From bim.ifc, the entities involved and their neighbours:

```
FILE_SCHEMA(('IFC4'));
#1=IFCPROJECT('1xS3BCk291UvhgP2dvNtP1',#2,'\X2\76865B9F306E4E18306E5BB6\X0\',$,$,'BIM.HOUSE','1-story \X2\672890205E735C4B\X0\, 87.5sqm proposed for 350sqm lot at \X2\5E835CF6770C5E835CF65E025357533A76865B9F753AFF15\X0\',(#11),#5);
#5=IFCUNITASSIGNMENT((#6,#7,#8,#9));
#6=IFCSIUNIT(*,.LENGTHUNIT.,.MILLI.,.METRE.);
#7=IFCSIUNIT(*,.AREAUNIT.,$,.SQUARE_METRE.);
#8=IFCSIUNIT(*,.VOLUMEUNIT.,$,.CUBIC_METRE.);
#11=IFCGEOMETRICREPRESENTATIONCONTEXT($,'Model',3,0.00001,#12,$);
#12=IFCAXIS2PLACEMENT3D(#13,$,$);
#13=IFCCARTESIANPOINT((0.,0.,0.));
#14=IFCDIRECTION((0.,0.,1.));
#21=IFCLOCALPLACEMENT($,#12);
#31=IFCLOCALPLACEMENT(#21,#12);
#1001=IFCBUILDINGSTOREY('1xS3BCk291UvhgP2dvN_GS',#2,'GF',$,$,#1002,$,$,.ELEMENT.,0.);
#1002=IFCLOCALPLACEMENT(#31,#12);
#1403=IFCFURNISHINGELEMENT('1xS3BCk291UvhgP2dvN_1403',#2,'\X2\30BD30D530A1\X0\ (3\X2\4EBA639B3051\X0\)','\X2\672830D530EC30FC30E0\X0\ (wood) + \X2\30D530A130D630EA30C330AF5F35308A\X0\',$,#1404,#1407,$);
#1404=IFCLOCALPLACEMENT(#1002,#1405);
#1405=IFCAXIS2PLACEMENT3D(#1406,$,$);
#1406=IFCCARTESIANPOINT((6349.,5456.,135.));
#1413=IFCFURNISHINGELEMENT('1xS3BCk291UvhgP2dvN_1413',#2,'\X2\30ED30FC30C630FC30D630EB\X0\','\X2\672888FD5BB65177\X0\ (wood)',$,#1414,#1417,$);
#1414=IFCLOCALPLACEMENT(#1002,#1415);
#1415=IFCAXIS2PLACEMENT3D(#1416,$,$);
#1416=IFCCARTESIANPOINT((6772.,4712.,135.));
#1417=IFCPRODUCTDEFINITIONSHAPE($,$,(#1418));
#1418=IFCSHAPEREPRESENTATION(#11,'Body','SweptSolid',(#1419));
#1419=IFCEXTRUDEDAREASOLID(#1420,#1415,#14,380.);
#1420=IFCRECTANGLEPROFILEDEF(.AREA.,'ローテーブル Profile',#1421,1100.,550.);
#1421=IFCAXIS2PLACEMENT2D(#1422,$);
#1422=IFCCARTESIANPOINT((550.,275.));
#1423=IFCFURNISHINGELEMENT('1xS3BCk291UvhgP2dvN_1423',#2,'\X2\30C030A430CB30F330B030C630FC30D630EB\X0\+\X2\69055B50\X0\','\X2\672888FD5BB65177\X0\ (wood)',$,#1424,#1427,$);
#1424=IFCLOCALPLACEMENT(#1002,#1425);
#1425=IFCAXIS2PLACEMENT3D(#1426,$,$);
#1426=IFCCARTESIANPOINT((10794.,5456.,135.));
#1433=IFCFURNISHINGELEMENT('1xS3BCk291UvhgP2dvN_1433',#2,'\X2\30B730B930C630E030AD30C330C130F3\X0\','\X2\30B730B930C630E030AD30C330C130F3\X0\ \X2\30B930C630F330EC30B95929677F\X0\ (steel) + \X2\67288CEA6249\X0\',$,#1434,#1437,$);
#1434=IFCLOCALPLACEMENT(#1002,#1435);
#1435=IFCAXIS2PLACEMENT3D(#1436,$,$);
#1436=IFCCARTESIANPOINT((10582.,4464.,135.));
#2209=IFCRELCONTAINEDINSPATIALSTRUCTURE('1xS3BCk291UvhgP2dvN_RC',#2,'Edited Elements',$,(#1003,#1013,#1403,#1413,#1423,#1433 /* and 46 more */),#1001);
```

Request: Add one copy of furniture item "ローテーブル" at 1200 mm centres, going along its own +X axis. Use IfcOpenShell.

```python
import ifcopenshell
import ifcopenshell.api.geometry
import ifcopenshell.api.root
import ifcopenshell.util.element
import ifcopenshell.util.placement

model = ifcopenshell.open("bim.ifc")


def reuse_history(source, copy):
    """copy_class also copies each property set's owner history, people and application; keep the originals."""
    for rel in copy.IsDefinedBy:
        if rel.is_a("IfcRelDefinesByProperties") and (history := rel.RelatingPropertyDefinition.OwnerHistory):
            rel.RelatingPropertyDefinition.OwnerHistory = source.OwnerHistory
            ifcopenshell.util.element.remove_deep2(model, history)


source = model.by_guid("1xS3BCk291UvhgP2dvN_1413")
base = ifcopenshell.util.placement.get_local_placement(source.ObjectPlacement)
step = base[:3, 0] * 1200.0

for i in range(1, 2):
    copy = ifcopenshell.api.root.copy_class(model, product=source)
    copy.Representation = ifcopenshell.util.element.copy_deep(
        model, source.Representation, exclude=["IfcGeometricRepresentationContext", "IfcRepresentationMap"]
    )
    reuse_history(source, copy)
    matrix = base.copy()
    matrix[:3, 3] += i * step
    print("added at", matrix[:3, 3].round(3) + 0.0)
    ifcopenshell.api.geometry.edit_object_placement(model, product=copy, matrix=matrix, is_si=False)

model.write("bim_rev.ifc")
```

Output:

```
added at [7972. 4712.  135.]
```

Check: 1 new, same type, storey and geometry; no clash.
